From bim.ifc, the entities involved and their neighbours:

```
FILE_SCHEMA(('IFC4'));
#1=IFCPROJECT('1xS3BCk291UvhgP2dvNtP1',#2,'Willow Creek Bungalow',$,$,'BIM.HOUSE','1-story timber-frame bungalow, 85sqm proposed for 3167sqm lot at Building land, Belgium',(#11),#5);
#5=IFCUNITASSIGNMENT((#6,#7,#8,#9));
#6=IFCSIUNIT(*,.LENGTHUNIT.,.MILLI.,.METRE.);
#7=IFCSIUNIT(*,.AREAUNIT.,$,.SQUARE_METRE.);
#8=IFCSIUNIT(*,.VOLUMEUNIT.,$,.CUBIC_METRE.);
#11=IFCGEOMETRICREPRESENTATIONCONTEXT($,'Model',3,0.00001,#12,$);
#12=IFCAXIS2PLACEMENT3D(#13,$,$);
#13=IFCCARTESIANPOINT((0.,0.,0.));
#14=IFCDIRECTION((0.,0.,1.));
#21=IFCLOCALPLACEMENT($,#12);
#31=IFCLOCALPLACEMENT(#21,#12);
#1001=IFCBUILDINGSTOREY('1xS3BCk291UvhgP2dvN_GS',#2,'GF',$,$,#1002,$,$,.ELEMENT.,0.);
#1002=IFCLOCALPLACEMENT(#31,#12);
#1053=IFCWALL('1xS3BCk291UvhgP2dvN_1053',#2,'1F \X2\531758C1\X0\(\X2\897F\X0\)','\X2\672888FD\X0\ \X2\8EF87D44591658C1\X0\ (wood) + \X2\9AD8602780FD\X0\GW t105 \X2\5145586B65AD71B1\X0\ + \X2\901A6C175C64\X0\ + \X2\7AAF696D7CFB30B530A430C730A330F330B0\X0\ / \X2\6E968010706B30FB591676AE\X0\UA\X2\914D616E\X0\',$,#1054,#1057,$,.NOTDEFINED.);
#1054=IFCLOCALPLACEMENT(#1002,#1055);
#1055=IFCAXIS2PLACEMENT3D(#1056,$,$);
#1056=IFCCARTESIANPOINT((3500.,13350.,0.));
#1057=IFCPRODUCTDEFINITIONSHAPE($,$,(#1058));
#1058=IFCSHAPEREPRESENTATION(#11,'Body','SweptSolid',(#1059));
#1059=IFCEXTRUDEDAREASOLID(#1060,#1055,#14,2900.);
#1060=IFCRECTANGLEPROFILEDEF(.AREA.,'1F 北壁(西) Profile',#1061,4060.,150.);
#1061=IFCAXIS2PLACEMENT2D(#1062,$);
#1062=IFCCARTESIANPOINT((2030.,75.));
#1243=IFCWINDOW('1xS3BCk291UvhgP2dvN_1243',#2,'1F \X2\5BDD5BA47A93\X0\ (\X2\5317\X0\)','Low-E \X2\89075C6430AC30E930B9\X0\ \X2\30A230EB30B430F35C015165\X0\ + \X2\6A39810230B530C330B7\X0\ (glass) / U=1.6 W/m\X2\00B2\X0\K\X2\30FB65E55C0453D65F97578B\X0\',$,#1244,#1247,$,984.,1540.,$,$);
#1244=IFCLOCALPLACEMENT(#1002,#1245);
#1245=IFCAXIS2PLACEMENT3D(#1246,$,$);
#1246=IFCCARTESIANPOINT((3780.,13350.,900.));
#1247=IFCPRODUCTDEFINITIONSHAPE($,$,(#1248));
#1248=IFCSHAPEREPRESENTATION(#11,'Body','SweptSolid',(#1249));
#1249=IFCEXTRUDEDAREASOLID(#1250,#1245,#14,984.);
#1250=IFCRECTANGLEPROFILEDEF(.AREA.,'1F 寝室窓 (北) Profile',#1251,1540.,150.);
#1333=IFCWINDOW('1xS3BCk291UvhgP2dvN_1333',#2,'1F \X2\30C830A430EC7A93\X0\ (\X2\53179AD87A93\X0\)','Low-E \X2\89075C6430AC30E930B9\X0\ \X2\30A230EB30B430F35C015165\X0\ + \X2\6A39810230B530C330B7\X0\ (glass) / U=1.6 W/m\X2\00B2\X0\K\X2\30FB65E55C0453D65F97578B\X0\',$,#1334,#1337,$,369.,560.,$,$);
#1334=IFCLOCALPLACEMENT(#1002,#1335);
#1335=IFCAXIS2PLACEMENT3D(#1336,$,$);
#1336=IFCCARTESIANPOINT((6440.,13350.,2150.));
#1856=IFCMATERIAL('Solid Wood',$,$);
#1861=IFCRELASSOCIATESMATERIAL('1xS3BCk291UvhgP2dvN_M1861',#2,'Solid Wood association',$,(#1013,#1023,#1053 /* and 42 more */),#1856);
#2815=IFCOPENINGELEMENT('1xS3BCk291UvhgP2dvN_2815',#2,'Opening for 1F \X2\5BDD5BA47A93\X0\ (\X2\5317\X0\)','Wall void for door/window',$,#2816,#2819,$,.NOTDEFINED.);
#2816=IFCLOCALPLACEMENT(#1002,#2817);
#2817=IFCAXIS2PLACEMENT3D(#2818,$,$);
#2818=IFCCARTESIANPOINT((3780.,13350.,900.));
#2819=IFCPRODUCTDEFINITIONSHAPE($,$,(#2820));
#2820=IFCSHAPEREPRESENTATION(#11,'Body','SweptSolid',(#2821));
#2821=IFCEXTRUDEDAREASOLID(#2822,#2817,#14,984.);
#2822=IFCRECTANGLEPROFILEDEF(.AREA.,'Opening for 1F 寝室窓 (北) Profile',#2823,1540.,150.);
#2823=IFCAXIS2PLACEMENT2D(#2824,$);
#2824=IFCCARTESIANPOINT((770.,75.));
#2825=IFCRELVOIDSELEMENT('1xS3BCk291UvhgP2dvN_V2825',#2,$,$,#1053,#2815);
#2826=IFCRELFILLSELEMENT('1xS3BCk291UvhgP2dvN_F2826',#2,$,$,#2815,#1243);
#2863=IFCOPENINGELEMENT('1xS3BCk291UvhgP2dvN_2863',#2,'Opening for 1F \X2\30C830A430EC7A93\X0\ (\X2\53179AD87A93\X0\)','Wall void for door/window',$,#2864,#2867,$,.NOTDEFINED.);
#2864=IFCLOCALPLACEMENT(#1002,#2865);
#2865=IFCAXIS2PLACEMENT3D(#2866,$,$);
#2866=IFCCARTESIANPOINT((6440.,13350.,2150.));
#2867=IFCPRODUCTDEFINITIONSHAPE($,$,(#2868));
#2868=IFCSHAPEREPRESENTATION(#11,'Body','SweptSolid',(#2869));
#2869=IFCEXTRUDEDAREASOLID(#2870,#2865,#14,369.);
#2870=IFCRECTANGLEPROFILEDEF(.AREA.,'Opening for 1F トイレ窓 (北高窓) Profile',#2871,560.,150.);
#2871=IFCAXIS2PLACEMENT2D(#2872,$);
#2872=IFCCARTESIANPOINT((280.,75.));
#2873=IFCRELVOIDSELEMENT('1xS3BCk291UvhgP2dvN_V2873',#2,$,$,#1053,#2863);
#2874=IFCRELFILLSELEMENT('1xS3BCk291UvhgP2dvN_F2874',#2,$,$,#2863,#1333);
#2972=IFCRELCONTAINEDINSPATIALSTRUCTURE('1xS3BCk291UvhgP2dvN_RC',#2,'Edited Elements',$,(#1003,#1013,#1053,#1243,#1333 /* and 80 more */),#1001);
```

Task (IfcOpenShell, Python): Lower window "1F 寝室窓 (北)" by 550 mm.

```python
import numpy as np
import ifcopenshell
import ifcopenshell.api.geometry
import ifcopenshell.util.placement
import ifcopenshell.util.unit

model = ifcopenshell.open("bim.ifc")
unit_scale = ifcopenshell.util.unit.calculate_unit_scale(model)

window = model.by_guid("1xS3BCk291UvhgP2dvN_1243")
opening = window.FillsVoids[0].RelatingOpeningElement
dz = -550.0

shift = np.array([0.0, 0.0, dz])
# The window is not placed relative to its opening, so move both.
for product in (opening, window):
    matrix = ifcopenshell.util.placement.get_local_placement(product.ObjectPlacement)
    matrix[:3, 3] += shift
    ifcopenshell.api.geometry.edit_object_placement(model, product=product, matrix=matrix, is_si=False)

print(f"moved by {dz * unit_scale:+.3f} m")

model.write("bim_rev.ifc")
```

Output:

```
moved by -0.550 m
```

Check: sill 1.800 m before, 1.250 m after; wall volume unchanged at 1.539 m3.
